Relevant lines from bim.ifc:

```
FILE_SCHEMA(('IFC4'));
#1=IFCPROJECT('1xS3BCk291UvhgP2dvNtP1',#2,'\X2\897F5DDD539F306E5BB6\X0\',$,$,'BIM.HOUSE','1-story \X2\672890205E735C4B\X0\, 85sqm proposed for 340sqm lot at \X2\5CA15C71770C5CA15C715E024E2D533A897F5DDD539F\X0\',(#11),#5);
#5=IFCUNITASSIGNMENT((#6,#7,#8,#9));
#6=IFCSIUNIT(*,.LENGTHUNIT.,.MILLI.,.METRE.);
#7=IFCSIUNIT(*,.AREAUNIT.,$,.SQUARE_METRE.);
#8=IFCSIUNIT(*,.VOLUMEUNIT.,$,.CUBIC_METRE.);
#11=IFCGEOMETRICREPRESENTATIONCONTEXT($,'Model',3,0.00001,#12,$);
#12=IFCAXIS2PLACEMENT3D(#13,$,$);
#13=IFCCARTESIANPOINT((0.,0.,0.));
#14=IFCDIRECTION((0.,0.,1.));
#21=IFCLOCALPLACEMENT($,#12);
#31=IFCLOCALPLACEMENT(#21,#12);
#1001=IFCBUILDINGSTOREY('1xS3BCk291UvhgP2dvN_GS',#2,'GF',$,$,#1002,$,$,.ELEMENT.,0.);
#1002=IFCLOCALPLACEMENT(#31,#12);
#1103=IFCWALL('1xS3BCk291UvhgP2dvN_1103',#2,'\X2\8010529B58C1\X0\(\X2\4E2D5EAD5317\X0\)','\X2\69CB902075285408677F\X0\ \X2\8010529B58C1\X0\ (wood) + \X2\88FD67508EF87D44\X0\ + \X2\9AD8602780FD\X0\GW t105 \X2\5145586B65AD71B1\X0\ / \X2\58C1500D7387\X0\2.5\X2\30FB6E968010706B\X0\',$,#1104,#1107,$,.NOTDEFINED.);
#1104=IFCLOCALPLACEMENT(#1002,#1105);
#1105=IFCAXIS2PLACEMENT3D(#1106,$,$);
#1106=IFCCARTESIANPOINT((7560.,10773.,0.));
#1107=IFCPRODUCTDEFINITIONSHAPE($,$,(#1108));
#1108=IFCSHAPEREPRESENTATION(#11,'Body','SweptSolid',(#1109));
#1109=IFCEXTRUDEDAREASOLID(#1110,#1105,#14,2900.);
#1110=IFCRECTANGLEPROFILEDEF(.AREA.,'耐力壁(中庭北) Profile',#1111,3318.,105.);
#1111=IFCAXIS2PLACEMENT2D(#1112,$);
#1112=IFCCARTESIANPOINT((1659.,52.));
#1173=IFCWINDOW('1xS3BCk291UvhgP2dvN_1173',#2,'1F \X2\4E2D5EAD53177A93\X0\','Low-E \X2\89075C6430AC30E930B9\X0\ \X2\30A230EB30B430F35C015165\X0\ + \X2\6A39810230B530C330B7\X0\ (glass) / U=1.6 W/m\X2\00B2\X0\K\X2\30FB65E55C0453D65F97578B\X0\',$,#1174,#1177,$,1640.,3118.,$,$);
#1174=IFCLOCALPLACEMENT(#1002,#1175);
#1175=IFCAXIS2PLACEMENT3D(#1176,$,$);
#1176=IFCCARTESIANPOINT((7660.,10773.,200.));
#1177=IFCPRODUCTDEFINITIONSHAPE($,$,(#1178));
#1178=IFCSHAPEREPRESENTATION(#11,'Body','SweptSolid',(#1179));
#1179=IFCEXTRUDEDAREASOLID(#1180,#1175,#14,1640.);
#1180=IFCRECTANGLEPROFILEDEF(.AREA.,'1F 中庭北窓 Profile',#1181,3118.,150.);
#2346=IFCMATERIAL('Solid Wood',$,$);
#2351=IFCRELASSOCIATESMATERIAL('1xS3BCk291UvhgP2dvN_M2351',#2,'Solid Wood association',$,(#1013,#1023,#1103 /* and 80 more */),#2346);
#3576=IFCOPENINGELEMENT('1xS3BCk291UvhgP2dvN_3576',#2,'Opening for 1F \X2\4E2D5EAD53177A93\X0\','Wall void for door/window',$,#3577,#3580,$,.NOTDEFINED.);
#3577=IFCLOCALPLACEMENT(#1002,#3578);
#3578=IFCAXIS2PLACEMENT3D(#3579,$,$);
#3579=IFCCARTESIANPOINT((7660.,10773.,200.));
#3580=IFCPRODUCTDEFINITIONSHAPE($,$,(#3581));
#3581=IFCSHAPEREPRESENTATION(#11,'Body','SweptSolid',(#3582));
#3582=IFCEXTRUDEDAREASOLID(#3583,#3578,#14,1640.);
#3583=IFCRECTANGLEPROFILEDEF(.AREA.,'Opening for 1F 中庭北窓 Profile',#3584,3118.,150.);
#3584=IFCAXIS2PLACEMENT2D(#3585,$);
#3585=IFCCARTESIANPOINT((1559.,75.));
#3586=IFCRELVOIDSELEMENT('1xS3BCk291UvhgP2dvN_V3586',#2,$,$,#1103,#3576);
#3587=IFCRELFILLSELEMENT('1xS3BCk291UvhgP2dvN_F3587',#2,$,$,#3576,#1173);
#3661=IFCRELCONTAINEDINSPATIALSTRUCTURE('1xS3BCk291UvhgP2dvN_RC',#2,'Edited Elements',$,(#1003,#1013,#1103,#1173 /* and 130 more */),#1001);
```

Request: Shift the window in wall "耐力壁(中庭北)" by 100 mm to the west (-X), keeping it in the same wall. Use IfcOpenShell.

```python
import ifcopenshell
import ifcopenshell.api.geometry
import ifcopenshell.util.placement

model = ifcopenshell.open("bim.ifc")

window = model.by_guid("1xS3BCk291UvhgP2dvN_1173")
opening = window.FillsVoids[0].RelatingOpeningElement
wall = opening.VoidsElements[0].RelatingBuildingElement

wall_matrix = ifcopenshell.util.placement.get_local_placement(wall.ObjectPlacement)
shift = wall_matrix[:3, 0] * -100.0
before = ifcopenshell.util.placement.get_local_placement(window.ObjectPlacement)[:3, 3].copy()

# The window is not placed relative to its opening, so move both.
for product in (opening, window):
    matrix = ifcopenshell.util.placement.get_local_placement(product.ObjectPlacement)
    matrix[:3, 3] += shift
    ifcopenshell.api.geometry.edit_object_placement(model, product=product, matrix=matrix, is_si=False)

after = ifcopenshell.util.placement.get_local_placement(window.ObjectPlacement)[:3, 3]
print("window moved by", (after - before).round(3) + 0.0)

model.write("bim_updated.ifc")
```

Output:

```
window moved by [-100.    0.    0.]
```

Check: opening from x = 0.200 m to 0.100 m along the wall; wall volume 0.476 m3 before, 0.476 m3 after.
